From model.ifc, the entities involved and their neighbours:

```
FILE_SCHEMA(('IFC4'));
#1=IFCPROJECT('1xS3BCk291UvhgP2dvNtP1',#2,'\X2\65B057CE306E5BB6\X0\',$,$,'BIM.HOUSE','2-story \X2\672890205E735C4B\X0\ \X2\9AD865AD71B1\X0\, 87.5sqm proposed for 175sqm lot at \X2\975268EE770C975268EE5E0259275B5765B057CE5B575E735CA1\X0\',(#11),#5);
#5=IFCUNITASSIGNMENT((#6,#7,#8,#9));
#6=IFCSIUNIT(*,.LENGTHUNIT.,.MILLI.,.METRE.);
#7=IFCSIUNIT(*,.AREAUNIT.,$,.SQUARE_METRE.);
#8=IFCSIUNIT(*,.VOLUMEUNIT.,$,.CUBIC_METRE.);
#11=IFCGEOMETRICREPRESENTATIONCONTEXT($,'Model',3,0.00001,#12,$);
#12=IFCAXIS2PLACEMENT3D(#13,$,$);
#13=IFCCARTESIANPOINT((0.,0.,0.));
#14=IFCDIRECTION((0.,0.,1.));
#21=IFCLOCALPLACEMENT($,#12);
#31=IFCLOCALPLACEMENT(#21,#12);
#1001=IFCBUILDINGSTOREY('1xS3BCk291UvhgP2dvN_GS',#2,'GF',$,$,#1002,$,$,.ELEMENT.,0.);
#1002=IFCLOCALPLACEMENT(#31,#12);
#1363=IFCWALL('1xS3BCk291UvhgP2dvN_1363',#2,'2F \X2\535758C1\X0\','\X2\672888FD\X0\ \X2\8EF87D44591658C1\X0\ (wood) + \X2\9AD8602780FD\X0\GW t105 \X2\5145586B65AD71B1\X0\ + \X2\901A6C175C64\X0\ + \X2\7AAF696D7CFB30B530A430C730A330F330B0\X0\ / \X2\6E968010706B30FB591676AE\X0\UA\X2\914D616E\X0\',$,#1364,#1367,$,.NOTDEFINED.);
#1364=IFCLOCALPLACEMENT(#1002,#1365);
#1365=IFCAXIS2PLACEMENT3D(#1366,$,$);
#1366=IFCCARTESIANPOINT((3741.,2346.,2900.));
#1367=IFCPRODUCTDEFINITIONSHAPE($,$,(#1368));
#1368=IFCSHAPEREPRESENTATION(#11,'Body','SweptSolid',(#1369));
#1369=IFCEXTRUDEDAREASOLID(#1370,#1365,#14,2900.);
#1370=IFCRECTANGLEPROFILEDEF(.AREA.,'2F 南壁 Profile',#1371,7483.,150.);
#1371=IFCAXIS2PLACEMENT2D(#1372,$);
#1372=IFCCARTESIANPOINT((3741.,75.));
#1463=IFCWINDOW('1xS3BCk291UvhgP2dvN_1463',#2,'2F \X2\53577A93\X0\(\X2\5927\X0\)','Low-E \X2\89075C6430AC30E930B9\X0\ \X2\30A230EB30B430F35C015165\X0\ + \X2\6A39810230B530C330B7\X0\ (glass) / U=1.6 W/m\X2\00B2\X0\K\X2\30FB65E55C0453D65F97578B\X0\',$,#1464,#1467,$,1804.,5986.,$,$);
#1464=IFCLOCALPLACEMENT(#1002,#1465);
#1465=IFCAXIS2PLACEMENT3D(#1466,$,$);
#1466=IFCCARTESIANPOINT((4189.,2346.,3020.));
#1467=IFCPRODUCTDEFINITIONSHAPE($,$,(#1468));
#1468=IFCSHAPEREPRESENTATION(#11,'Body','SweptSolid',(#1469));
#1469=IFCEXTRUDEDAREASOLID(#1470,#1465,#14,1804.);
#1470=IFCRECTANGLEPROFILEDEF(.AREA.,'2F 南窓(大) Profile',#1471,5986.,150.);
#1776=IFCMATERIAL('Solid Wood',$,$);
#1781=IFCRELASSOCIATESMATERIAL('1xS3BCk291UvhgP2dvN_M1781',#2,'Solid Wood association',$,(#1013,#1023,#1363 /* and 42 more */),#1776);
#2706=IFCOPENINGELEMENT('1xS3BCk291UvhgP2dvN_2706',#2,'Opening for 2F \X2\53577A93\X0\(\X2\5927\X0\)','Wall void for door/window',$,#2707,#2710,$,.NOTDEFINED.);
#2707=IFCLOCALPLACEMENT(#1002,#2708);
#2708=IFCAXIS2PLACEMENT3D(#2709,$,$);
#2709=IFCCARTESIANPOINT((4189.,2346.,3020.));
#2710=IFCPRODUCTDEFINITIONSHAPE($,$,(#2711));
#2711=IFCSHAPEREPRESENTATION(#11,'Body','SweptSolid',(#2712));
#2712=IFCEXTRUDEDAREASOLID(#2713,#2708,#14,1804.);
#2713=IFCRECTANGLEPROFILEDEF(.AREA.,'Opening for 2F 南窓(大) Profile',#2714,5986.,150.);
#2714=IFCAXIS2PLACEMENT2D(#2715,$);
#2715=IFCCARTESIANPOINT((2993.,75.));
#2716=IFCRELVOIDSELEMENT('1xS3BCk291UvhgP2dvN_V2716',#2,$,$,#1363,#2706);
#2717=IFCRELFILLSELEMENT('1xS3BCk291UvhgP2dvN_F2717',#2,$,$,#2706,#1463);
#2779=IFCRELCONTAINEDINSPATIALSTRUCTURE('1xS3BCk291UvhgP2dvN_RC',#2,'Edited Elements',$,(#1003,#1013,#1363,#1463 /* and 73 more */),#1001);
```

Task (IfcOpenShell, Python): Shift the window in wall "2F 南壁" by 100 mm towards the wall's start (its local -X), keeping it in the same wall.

```python
import ifcopenshell
import ifcopenshell.api.geometry
import ifcopenshell.util.placement

model = ifcopenshell.open("model.ifc")

window = model.by_guid("1xS3BCk291UvhgP2dvN_1463")
opening = window.FillsVoids[0].RelatingOpeningElement
wall = opening.VoidsElements[0].RelatingBuildingElement

wall_matrix = ifcopenshell.util.placement.get_local_placement(wall.ObjectPlacement)
shift = wall_matrix[:3, 0] * -100.0
before = ifcopenshell.util.placement.get_local_placement(window.ObjectPlacement)[:3, 3].copy()

# The window is not placed relative to its opening, so move both.
for product in (opening, window):
    matrix = ifcopenshell.util.placement.get_local_placement(product.ObjectPlacement)
    matrix[:3, 3] += shift
    ifcopenshell.api.geometry.edit_object_placement(model, product=product, matrix=matrix, is_si=False)

after = ifcopenshell.util.placement.get_local_placement(window.ObjectPlacement)[:3, 3]
print("window moved by", (after - before).round(3) + 0.0)

model.write("model_rev.ifc")
```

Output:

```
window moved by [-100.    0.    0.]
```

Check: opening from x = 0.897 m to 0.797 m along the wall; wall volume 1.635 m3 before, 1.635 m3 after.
